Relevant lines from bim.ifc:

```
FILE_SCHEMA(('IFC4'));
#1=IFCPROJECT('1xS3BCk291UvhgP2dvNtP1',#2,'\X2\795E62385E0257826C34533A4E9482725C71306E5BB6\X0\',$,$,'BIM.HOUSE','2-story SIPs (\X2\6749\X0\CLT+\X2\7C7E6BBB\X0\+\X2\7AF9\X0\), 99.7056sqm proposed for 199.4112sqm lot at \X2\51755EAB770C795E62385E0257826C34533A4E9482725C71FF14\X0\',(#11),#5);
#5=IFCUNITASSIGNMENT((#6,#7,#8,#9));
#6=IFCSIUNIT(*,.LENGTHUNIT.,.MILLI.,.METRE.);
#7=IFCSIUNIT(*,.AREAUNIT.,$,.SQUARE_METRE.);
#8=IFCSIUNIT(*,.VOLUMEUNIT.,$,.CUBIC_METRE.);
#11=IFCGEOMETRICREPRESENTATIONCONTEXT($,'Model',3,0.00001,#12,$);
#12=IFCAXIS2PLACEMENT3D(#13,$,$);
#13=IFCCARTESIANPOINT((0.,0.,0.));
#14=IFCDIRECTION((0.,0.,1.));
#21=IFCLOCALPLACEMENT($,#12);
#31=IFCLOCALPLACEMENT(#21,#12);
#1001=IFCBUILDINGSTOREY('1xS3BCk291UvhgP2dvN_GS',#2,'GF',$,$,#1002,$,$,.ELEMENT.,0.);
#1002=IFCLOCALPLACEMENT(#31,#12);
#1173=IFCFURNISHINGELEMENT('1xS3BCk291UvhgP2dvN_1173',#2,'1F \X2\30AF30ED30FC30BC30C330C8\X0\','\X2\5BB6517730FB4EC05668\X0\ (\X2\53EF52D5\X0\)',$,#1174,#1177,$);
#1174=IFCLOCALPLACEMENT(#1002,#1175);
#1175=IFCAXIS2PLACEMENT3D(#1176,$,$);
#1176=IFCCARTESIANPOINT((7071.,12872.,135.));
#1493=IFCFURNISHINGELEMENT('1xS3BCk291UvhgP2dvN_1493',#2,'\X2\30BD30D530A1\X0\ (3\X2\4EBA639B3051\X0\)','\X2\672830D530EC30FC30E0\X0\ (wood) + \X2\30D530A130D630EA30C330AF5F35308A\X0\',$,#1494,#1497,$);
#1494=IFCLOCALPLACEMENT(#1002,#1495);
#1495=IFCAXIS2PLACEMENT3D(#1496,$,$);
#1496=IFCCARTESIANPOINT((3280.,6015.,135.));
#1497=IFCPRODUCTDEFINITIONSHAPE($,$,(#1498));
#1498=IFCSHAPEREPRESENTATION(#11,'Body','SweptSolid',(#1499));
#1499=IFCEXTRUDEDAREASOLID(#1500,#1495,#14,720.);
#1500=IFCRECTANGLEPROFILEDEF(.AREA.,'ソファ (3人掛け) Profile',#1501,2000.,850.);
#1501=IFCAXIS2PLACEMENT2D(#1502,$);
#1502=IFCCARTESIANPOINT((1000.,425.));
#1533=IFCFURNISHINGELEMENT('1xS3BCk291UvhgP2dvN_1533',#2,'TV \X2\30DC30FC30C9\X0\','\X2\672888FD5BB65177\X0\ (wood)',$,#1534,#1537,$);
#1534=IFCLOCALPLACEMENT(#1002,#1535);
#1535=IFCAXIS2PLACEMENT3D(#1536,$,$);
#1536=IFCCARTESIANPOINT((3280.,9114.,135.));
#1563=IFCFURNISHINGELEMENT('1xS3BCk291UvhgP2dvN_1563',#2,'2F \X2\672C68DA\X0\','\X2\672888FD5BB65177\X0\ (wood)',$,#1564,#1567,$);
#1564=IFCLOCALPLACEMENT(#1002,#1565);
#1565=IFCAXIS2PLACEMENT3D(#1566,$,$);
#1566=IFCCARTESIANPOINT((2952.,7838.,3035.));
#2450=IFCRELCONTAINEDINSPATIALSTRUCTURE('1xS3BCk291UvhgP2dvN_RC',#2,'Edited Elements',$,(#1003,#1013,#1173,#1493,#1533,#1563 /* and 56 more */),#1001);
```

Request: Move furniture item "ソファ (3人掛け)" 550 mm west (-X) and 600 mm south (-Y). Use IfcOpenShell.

```python
import ifcopenshell
import ifcopenshell.api.geometry
import ifcopenshell.util.placement

model = ifcopenshell.open("bim.ifc")

item = model.by_guid("1xS3BCk291UvhgP2dvN_1493")
matrix = ifcopenshell.util.placement.get_local_placement(item.ObjectPlacement)
matrix[0, 3] -= 550.0
matrix[1, 3] -= 600.0
ifcopenshell.api.geometry.edit_object_placement(model, product=item, matrix=matrix, is_si=False)

print(ifcopenshell.util.placement.get_local_placement(item.ObjectPlacement).round(3) + 0.0)

model.write("bim-out.ifc")
```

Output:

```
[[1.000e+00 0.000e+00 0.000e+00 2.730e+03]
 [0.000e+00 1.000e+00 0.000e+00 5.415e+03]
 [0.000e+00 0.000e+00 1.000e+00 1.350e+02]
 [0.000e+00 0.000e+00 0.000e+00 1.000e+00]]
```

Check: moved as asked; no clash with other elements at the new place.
